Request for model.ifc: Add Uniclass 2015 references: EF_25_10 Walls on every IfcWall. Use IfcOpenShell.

First a look at what the model holds.

```python
import ifcopenshell

model = ifcopenshell.open("model.ifc")
print(model.schema)
print("classifications:", [c.Name for c in model.by_type("IfcClassification")])
for ifc_class in ("IfcDoor", "IfcRoof", "IfcStair", "IfcWall", "IfcWindow"):
    print(ifc_class, len(model.by_type(ifc_class)))
```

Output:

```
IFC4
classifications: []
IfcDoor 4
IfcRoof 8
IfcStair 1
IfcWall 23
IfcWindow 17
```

```python
import ifcopenshell
import ifcopenshell.api.classification

model = ifcopenshell.open("model.ifc")

system = ifcopenshell.api.classification.add_classification(model, classification="Uniclass 2015")

codes = {
    "IfcWall": ("EF_25_10", "Walls"),
}
for ifc_class, (code, name) in codes.items():
    products = model.by_type(ifc_class)
    ifcopenshell.api.classification.add_reference(
        model, products=products, classification=system, identification=code, name=name
    )
    print(code, len(products))

model.write("model_v2.ifc")
```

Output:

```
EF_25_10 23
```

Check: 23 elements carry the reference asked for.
